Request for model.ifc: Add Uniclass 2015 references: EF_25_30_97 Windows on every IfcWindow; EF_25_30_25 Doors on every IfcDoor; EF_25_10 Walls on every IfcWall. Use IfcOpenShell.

First a look at what the model holds.

```python
import ifcopenshell

model = ifcopenshell.open("model.ifc")
print(model.schema)
print("classifications:", [c.Name for c in model.by_type("IfcClassification")])
for ifc_class in ("IfcDoor", "IfcRoof", "IfcStair", "IfcWall", "IfcWindow"):
    print(ifc_class, len(model.by_type(ifc_class)))
```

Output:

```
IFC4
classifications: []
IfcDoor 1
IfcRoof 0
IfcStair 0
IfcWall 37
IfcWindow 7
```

```python
import ifcopenshell
import ifcopenshell.api.classification

model = ifcopenshell.open("model.ifc")

system = ifcopenshell.api.classification.add_classification(model, classification="Uniclass 2015")

codes = {
    "IfcWindow": ("EF_25_30_97", "Windows"),
    "IfcDoor": ("EF_25_30_25", "Doors"),
    "IfcWall": ("EF_25_10", "Walls"),
}
for ifc_class, (code, name) in codes.items():
    products = model.by_type(ifc_class)
    ifcopenshell.api.classification.add_reference(
        model, products=products, classification=system, identification=code, name=name
    )
    print(code, len(products))

model.write("model_edited.ifc")
```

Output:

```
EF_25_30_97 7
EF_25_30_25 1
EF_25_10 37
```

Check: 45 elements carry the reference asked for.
